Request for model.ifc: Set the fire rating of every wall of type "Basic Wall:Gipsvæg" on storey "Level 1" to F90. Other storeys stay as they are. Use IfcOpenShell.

First a look at what the model holds.

```python
import ifcopenshell
import ifcopenshell.util.element

model = ifcopenshell.open("model.ifc")
print(model.schema)
storey = next(s for s in model.by_type("IfcBuildingStorey") if s.Name == "Level 1")
walls = [e for e in ifcopenshell.util.element.get_decomposition(storey) if e.is_a("IfcWall")]
seen = {}
for e in walls:
    element_type = ifcopenshell.util.element.get_type(e)
    key = (element_type.Name if element_type != e and element_type else None, ifcopenshell.util.element.get_pset(e, "Pset_WallCommon", "FireRating"))
    seen[key] = seen.get(key, 0) + 1
for (name, value), count in sorted(seen.items(), key=str):
    print(count, "x", name, "|", value)
```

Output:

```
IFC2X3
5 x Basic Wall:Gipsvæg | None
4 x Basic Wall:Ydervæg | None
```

```python
import ifcopenshell
import ifcopenshell.api.pset
import ifcopenshell.util.element

model = ifcopenshell.open("model.ifc")

storey = next(s for s in model.by_type("IfcBuildingStorey") if s.Name == "Level 1")
walls = [e for e in ifcopenshell.util.element.get_decomposition(storey) if e.is_a("IfcWall")]

count = 0
for e in walls:
    element_type = ifcopenshell.util.element.get_type(e)
    if element_type in (None, e) or element_type.Name != "Basic Wall:Gipsvæg":
        continue
    # add_pset returns the element's existing set when there is one.
    pset = ifcopenshell.api.pset.add_pset(model, product=e, name="Pset_WallCommon")
    ifcopenshell.api.pset.edit_pset(model, pset=pset, properties={"FireRating": "F90"})
    count += 1

print(count, "walls updated")

model.write("model_updated.ifc")
```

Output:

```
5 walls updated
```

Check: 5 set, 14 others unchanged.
